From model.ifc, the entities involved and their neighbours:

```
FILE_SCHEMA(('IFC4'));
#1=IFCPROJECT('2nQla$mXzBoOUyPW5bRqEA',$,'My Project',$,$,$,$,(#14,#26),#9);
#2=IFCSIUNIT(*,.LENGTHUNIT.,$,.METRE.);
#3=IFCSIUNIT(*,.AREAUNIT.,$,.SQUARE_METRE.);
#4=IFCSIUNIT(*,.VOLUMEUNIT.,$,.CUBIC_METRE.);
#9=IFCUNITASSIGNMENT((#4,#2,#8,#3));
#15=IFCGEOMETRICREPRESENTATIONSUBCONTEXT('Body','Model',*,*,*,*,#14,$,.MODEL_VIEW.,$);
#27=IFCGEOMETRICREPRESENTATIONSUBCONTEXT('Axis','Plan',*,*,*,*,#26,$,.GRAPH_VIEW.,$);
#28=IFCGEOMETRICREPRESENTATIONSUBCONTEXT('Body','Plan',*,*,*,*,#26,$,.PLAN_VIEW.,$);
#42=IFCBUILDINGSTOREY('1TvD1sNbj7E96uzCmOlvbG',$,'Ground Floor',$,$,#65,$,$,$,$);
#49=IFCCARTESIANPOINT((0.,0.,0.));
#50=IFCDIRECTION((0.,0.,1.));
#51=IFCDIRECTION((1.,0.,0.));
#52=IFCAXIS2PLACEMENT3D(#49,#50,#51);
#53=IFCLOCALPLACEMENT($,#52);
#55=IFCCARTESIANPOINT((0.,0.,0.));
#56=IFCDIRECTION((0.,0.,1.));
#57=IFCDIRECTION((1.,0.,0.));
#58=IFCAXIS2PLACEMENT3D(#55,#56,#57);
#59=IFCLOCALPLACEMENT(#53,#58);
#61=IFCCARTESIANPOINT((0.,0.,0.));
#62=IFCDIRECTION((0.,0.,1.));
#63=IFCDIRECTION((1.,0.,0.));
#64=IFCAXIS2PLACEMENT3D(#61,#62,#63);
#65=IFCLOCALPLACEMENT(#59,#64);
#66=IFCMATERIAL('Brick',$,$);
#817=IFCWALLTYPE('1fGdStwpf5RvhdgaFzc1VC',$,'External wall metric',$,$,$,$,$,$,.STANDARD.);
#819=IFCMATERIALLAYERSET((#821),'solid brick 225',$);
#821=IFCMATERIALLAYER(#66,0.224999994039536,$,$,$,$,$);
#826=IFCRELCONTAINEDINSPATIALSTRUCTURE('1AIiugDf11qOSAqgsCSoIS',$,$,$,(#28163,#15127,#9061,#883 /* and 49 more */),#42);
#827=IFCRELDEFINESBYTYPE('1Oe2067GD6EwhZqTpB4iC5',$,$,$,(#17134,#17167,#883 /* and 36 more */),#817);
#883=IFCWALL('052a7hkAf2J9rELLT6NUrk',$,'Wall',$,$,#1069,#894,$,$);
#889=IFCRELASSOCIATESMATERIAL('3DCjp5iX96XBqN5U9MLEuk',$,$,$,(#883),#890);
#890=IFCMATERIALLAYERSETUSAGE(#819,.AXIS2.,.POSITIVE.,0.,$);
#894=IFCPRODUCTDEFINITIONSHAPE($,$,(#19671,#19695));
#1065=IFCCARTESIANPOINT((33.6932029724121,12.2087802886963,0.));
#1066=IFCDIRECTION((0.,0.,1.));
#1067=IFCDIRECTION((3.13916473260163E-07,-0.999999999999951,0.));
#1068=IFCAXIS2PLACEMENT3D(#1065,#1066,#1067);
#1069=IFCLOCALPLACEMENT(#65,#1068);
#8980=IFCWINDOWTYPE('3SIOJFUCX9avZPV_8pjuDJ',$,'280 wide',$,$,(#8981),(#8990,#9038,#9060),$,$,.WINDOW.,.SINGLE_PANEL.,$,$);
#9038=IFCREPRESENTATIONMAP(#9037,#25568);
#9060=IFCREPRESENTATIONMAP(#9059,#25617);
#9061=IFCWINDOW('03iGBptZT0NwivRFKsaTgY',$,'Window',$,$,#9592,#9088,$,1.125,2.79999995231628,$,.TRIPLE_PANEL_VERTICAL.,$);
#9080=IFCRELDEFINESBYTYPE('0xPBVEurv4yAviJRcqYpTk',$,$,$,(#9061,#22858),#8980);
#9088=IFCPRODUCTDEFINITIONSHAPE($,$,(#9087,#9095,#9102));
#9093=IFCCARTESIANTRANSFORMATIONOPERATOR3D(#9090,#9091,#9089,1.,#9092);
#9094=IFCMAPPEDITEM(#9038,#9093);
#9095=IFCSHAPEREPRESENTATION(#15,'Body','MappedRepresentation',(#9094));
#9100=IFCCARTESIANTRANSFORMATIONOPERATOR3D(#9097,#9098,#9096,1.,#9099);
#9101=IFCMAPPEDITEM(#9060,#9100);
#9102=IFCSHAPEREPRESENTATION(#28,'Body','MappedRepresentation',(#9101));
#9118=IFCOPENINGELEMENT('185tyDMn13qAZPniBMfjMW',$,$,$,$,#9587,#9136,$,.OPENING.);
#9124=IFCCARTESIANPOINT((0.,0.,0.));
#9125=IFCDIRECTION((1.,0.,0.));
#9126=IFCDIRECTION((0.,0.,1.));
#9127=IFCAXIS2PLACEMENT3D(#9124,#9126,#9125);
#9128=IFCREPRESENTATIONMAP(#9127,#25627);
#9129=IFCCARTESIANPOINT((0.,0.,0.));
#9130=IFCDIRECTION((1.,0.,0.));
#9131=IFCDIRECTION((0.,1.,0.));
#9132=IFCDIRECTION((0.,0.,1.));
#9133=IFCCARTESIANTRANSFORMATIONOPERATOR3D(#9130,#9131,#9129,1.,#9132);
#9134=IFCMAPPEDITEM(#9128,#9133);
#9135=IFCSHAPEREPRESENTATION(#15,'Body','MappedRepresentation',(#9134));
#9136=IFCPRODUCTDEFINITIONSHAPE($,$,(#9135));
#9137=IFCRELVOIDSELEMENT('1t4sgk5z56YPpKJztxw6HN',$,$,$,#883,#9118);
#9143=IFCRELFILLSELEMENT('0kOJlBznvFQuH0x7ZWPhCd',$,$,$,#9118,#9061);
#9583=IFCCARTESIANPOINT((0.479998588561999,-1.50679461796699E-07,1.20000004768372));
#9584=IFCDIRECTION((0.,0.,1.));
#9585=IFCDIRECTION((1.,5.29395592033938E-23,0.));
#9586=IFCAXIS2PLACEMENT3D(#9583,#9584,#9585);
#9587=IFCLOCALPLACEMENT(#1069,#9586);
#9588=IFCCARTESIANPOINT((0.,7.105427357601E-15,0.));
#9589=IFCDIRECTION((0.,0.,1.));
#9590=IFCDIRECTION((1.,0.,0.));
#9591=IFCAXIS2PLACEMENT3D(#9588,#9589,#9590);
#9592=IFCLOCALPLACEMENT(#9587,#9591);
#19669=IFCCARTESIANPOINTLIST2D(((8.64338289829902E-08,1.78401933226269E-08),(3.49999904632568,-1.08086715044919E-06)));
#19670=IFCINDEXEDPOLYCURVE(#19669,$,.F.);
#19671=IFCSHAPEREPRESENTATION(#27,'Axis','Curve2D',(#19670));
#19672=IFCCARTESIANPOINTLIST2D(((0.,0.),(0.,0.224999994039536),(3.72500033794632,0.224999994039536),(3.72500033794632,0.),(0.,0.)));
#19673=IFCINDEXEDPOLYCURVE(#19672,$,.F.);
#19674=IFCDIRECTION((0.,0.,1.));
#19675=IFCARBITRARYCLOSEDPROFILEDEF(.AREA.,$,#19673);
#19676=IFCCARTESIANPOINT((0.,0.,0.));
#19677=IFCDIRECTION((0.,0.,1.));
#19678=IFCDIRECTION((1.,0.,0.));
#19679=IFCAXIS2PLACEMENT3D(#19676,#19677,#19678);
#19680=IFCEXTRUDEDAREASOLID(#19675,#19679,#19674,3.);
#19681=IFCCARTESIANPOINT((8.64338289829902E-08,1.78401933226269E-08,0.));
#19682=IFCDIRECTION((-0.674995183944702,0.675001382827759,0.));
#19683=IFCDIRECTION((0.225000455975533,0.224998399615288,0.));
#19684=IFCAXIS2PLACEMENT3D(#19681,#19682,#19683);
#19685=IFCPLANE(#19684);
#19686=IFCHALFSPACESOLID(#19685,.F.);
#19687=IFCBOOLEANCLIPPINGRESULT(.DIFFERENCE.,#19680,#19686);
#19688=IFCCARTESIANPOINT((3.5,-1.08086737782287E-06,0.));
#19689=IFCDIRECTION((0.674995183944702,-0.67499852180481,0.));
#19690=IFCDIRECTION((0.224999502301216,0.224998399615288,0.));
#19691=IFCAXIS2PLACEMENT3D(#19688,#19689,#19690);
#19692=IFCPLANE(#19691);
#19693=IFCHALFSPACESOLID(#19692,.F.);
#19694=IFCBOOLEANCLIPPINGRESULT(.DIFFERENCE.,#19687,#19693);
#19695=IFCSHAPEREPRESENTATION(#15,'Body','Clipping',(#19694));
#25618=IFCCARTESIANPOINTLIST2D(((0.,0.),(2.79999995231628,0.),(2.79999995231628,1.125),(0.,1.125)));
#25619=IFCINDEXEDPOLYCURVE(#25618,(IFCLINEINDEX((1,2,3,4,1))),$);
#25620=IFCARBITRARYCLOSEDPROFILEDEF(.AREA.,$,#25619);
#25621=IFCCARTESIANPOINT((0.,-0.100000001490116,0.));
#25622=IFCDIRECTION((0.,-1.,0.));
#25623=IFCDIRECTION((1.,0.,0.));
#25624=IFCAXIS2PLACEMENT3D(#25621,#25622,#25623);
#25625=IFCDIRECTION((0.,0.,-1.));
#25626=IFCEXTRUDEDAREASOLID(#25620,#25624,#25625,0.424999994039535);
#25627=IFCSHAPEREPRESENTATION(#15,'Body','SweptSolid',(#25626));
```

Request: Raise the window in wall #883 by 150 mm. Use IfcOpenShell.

```python
import numpy as np
import ifcopenshell
import ifcopenshell.api.geometry
import ifcopenshell.util.placement
import ifcopenshell.util.unit

model = ifcopenshell.open("model.ifc")
unit_scale = ifcopenshell.util.unit.calculate_unit_scale(model)

window = model.by_guid("03iGBptZT0NwivRFKsaTgY")
opening = window.FillsVoids[0].RelatingOpeningElement
dz = 0.15 / unit_scale

shift = np.array([0.0, 0.0, dz])
# The window is placed relative to its opening, so it follows when the opening moves.
matrix = ifcopenshell.util.placement.get_local_placement(opening.ObjectPlacement)
matrix[:3, 3] += shift
ifcopenshell.api.geometry.edit_object_placement(
    model, product=opening, matrix=matrix, is_si=False, should_transform_children=True
)

print(f"moved by {dz * unit_scale:+.3f} m")

model.write("model_v2.ifc")
```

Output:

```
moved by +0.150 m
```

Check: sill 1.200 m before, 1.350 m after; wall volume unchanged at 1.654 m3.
